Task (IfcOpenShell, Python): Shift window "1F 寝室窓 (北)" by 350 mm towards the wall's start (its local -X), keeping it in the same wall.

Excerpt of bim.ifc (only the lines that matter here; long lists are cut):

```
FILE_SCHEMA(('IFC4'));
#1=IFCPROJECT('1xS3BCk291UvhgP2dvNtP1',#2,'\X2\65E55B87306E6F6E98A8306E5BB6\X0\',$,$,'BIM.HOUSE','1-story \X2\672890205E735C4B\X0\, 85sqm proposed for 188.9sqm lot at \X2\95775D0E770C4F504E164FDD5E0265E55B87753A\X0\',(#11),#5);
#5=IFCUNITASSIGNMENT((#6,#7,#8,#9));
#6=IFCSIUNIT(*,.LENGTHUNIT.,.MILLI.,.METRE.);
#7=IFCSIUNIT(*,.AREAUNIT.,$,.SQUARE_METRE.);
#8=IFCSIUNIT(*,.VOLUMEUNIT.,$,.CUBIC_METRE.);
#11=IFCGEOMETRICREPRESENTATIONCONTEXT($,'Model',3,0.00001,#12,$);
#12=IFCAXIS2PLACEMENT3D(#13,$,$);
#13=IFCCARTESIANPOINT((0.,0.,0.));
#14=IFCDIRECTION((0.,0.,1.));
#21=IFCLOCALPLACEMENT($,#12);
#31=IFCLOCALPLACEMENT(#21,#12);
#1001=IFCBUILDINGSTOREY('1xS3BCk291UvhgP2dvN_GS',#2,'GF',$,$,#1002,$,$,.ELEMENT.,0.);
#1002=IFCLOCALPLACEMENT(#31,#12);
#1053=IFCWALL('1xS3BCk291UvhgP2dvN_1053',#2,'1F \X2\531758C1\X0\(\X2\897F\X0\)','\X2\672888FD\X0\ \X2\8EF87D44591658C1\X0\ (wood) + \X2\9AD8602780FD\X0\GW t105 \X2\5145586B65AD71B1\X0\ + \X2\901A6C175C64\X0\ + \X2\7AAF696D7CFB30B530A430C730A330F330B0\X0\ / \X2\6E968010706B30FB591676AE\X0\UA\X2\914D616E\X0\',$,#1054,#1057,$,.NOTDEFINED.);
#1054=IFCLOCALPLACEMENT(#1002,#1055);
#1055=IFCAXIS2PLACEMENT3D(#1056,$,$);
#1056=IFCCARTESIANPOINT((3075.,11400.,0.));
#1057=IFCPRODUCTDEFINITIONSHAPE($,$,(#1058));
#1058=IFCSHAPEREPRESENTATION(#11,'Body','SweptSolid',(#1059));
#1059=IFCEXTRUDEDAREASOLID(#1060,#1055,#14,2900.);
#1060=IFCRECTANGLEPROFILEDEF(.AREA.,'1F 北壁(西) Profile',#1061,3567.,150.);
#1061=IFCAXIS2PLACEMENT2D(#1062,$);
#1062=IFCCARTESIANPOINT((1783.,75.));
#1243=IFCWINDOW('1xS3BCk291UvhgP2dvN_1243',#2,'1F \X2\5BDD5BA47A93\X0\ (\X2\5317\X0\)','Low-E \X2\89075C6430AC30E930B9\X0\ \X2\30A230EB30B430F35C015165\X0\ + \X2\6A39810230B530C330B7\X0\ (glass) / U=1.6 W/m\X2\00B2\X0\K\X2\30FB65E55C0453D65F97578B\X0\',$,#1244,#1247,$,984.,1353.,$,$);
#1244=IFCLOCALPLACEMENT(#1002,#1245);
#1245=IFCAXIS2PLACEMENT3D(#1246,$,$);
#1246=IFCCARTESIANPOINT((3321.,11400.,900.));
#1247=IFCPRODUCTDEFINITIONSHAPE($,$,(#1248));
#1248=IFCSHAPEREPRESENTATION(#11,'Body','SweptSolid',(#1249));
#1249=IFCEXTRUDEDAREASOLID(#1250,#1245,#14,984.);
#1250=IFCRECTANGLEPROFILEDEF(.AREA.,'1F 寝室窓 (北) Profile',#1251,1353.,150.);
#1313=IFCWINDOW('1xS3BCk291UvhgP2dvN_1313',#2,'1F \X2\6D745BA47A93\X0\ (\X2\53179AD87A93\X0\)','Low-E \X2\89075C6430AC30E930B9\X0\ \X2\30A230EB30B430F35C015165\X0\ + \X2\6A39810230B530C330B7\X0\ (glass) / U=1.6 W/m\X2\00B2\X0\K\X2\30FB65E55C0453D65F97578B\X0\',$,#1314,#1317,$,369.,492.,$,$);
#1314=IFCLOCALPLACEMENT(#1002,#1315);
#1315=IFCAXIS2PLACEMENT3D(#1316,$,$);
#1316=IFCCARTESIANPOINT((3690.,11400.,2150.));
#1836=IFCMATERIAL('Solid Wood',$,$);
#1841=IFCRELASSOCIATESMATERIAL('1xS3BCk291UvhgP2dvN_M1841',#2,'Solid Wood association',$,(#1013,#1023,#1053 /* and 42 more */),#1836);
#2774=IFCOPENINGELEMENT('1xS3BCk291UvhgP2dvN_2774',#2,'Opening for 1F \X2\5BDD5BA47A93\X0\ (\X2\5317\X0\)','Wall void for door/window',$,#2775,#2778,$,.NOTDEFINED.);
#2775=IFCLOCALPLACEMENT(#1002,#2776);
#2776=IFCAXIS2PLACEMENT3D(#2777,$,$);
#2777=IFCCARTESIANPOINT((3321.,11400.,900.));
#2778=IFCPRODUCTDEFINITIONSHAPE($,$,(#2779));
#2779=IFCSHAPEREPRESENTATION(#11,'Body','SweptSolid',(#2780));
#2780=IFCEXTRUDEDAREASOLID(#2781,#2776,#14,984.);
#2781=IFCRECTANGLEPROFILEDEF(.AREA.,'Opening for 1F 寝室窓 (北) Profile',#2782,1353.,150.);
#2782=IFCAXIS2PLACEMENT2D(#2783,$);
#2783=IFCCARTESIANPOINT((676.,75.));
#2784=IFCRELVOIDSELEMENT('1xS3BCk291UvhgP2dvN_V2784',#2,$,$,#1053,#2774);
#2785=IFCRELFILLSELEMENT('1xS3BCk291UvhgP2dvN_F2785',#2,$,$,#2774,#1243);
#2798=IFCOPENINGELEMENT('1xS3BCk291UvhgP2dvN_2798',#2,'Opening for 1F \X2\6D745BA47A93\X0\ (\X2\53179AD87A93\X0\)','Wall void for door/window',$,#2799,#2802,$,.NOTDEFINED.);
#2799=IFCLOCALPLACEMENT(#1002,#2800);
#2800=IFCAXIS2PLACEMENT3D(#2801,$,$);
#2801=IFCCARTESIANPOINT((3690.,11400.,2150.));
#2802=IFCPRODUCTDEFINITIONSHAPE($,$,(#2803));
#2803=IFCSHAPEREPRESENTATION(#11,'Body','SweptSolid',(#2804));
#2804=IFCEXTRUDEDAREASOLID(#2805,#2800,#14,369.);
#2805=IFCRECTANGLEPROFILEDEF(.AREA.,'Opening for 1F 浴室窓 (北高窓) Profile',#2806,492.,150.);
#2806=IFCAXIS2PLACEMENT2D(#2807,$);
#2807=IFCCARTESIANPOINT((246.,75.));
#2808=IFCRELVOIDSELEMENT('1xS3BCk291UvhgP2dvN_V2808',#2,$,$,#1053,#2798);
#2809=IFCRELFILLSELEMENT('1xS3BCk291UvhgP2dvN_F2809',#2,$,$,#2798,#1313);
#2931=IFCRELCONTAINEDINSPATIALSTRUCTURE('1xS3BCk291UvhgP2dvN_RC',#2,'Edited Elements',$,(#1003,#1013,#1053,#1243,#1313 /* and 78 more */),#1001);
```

```python
import ifcopenshell
import ifcopenshell.api.geometry
import ifcopenshell.util.placement
import ifcopenshell.util.unit

model = ifcopenshell.open("bim.ifc")
unit_scale = ifcopenshell.util.unit.calculate_unit_scale(model)

window = model.by_guid("1xS3BCk291UvhgP2dvN_1243")
opening = window.FillsVoids[0].RelatingOpeningElement
wall = opening.VoidsElements[0].RelatingBuildingElement

wall_matrix = ifcopenshell.util.placement.get_local_placement(wall.ObjectPlacement)
shift = wall_matrix[:3, 0] * -0.35 / unit_scale
before = ifcopenshell.util.placement.get_local_placement(window.ObjectPlacement)[:3, 3].copy()

# The window is not placed relative to its opening, so move both.
for product in (opening, window):
    matrix = ifcopenshell.util.placement.get_local_placement(product.ObjectPlacement)
    matrix[:3, 3] += shift
    ifcopenshell.api.geometry.edit_object_placement(model, product=product, matrix=matrix, is_si=False)

after = ifcopenshell.util.placement.get_local_placement(window.ObjectPlacement)[:3, 3]
print("window moved by", (after - before).round(3) + 0.0)

model.write("bim_updated.ifc")
```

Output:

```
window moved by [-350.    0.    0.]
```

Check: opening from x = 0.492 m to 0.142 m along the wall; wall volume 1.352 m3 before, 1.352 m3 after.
